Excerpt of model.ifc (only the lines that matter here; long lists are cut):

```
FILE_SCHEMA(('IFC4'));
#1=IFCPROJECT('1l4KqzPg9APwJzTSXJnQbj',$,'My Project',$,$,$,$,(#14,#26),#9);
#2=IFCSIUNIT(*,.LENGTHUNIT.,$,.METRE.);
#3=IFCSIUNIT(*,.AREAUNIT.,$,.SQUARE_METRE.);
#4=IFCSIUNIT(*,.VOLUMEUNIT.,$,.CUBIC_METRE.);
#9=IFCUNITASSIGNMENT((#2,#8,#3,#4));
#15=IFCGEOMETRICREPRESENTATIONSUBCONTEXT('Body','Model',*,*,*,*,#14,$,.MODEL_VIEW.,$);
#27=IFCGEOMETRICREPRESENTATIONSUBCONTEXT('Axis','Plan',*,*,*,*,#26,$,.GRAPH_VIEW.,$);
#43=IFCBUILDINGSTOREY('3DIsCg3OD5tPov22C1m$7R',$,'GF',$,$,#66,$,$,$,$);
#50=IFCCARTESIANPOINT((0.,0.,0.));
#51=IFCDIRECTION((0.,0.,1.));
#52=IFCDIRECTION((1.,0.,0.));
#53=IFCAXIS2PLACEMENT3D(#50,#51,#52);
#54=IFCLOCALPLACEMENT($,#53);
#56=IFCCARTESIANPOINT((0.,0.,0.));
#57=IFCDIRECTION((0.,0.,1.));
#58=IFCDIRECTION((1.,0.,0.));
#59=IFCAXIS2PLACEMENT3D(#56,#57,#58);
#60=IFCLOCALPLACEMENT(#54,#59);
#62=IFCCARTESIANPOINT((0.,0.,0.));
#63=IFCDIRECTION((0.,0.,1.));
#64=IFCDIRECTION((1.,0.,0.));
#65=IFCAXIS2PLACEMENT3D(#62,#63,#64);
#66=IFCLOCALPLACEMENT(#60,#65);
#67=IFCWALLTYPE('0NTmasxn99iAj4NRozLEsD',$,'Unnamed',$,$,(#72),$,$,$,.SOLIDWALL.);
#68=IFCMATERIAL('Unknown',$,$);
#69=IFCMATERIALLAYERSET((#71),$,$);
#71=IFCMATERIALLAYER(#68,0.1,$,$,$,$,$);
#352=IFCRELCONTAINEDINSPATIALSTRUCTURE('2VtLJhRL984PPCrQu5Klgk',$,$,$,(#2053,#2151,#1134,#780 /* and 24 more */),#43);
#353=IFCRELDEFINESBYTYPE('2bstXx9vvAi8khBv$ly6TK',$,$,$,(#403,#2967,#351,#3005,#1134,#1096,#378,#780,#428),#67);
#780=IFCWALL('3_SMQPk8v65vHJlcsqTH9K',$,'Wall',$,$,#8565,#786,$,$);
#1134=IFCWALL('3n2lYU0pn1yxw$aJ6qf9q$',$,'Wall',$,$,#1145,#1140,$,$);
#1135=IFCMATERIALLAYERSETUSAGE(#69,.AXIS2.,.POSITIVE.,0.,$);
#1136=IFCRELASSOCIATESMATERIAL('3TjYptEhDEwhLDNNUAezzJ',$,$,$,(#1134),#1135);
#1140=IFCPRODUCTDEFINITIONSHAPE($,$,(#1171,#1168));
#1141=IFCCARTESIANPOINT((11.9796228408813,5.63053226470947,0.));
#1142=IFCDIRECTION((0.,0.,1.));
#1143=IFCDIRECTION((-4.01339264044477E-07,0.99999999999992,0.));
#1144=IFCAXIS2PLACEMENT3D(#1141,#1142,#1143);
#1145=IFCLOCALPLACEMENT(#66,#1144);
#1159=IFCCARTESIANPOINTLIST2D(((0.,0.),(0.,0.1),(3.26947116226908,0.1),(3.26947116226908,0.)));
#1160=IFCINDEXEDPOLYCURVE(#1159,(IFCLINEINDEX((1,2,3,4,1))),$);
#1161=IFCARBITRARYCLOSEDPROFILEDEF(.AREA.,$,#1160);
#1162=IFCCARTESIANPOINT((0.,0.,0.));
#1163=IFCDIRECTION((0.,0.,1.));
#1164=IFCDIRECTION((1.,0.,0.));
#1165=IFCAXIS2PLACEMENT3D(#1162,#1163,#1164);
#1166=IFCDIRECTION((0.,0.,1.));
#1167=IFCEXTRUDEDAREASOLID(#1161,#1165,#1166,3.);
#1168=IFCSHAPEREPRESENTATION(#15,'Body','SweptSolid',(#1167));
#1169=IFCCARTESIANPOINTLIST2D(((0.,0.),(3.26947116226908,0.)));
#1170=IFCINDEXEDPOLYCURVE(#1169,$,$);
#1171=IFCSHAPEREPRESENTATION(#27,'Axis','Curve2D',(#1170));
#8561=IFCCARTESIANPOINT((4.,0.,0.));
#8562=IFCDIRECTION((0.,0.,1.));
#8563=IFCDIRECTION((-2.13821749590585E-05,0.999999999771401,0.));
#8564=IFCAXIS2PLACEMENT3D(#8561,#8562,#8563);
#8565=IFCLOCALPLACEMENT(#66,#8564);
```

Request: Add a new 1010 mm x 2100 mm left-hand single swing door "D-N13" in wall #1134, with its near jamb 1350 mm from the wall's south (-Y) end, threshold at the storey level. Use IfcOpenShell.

```python
import numpy as np
import ifcopenshell
import ifcopenshell.api.feature
import ifcopenshell.api.geometry
import ifcopenshell.api.root
import ifcopenshell.api.spatial
import ifcopenshell.geom
import ifcopenshell.util.element
import ifcopenshell.util.placement
import ifcopenshell.util.representation
import ifcopenshell.util.shape
import ifcopenshell.util.unit

model = ifcopenshell.open("model.ifc")
unit_scale = ifcopenshell.util.unit.calculate_unit_scale(model)
settings = ifcopenshell.geom.settings()


def volume(element):
    """Net volume in cubic metres, openings subtracted."""
    shape = ifcopenshell.geom.create_shape(settings, element)
    return ifcopenshell.util.shape.get_volume(shape.geometry)


wall = model.by_guid("3n2lYU0pn1yxw$aJ6qf9q$")
storey = ifcopenshell.util.element.get_container(wall, ifc_class="IfcBuildingStorey")
context = ifcopenshell.util.representation.get_context(model, "Model", "Body", "MODEL_VIEW")
before = volume(wall)

width, height, from_end, sill = 1.01, 2.1, 1.35, 0.0  # metres

# The wall runs along its own X axis, and the end named is its -X end.
wall_shape = ifcopenshell.geom.create_shape(settings, wall)
x, y, z = ifcopenshell.util.shape.get_vertices(wall_shape.geometry).T
start = x.min() + from_end
face, thickness = float(y.min()), float(y.max() - y.min())
wall_matrix = ifcopenshell.util.placement.get_local_placement(wall.ObjectPlacement)
level = ifcopenshell.util.placement.get_local_placement(storey.ObjectPlacement)[2, 3]


def in_wall(x, y):
    """Placement at x, y metres in the wall's axes, at sill height."""
    matrix = wall_matrix.copy()
    matrix[:, 3] = wall_matrix @ np.array([x / unit_scale, y / unit_scale, 0.0, 1.0])
    matrix[2, 3] = level + sill / unit_scale
    return matrix


# Opening: a box that overshoots both wall faces by 50 mm.
opening = ifcopenshell.api.root.create_entity(model, ifc_class="IfcOpeningElement", predefined_type="OPENING")
box = ifcopenshell.api.geometry.add_wall_representation(
    model, context=context, length=width, height=height, thickness=thickness + 0.1
)
ifcopenshell.api.geometry.assign_representation(model, product=opening, representation=box)
ifcopenshell.api.geometry.edit_object_placement(model, product=opening, matrix=in_wall(start, face - 0.05), is_si=False)
ifcopenshell.api.feature.add_feature(model, feature=opening, element=wall)

door = ifcopenshell.api.root.create_entity(model, ifc_class="IfcDoor", name="D-N13", predefined_type="DOOR")
door.OverallWidth, door.OverallHeight = width / unit_scale, height / unit_scale
door.OperationType = "SINGLE_SWING_LEFT"
body = ifcopenshell.api.geometry.add_door_representation(
    model,
    context=context,
    overall_width=door.OverallWidth,
    overall_height=door.OverallHeight,
    operation_type="SINGLE_SWING_LEFT",
    lining_properties={"LiningDepth": thickness / unit_scale, "ThresholdDepth": thickness / unit_scale},
)
ifcopenshell.api.geometry.assign_representation(model, product=door, representation=body)
ifcopenshell.api.spatial.assign_container(model, products=[door], relating_structure=storey)
ifcopenshell.api.feature.add_filling(model, opening=opening, element=door)

# The lining spans the wall, so the door starts at the wall face.
ifcopenshell.api.geometry.edit_object_placement(model, product=door, matrix=in_wall(start, face), is_si=False)

after = volume(wall)

print(f"wall volume {before:.3f} -> {after:.3f} m3")

model.write("model_v2.ifc")
```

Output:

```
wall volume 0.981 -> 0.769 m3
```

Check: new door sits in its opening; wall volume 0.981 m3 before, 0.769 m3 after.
